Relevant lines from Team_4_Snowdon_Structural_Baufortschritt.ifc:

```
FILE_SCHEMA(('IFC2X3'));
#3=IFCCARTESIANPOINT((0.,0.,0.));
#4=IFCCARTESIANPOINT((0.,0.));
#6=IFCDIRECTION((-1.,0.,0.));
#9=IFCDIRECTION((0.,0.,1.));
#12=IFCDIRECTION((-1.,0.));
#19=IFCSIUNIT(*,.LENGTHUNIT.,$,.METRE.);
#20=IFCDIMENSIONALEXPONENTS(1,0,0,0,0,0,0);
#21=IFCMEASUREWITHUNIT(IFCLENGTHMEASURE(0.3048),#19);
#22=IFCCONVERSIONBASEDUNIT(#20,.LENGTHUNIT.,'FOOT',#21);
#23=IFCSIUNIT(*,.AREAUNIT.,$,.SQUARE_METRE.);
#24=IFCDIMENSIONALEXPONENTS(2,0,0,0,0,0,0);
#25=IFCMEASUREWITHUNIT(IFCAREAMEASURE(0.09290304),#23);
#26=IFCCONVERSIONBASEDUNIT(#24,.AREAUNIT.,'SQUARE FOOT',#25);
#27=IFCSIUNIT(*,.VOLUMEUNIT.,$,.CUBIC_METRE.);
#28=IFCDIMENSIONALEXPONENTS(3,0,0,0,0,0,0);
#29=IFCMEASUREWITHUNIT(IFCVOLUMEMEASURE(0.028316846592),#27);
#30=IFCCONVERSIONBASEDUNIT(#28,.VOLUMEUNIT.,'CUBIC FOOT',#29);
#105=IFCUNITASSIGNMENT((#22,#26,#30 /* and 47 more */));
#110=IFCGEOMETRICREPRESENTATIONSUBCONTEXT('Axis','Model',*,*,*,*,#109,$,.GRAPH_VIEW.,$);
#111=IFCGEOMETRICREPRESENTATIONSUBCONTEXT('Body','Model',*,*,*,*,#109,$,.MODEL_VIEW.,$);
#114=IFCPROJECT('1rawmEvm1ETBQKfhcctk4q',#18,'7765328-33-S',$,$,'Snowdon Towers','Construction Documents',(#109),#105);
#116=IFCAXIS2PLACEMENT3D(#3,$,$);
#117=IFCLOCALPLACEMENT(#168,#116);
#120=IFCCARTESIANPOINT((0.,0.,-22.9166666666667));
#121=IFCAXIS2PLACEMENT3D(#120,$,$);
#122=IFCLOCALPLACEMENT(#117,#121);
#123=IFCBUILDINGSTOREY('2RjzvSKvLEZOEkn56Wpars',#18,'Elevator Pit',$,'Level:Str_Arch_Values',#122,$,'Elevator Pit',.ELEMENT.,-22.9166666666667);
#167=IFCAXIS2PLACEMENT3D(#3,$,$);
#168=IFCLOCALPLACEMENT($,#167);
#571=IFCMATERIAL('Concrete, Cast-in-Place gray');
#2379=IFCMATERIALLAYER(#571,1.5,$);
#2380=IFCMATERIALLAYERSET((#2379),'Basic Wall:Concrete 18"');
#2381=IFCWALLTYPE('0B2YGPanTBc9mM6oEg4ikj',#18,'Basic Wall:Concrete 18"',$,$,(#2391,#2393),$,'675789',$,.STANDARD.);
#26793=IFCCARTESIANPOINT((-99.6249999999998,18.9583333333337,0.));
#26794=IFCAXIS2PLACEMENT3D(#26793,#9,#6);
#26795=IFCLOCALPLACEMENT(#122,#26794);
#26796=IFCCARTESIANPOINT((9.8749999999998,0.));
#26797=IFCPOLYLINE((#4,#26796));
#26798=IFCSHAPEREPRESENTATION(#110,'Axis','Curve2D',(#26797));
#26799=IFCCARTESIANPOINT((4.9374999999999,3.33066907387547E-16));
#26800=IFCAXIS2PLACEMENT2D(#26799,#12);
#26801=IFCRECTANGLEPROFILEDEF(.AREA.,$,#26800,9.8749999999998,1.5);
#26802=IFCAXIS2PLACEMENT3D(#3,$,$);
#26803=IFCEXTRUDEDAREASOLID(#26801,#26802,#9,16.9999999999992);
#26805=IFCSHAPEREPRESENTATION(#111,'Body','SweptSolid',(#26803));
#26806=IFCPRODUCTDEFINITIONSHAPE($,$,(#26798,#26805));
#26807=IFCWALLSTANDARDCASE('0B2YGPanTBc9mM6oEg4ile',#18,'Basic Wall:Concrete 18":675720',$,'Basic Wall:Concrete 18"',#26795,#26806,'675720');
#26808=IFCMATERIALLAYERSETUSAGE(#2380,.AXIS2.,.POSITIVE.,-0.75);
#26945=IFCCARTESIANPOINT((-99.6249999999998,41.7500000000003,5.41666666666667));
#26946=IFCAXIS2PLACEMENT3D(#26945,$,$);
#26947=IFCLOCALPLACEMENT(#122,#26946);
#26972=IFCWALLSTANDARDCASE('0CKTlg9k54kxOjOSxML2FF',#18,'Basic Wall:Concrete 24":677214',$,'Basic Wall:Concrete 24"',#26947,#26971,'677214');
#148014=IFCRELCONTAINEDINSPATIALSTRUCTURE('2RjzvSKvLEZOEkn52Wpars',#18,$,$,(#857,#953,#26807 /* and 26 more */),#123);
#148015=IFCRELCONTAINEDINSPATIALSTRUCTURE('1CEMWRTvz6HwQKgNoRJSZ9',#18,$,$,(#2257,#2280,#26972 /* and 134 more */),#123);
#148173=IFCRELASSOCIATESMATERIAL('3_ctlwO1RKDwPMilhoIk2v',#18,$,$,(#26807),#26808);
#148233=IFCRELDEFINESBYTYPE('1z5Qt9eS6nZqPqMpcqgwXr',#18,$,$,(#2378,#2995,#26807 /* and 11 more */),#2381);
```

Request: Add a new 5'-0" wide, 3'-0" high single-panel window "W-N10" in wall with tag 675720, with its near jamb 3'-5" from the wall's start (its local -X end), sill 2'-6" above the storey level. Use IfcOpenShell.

```python
import numpy as np
import ifcopenshell
import ifcopenshell.api.feature
import ifcopenshell.api.geometry
import ifcopenshell.api.root
import ifcopenshell.api.spatial
import ifcopenshell.api.type
import ifcopenshell.geom
import ifcopenshell.util.element
import ifcopenshell.util.placement
import ifcopenshell.util.representation
import ifcopenshell.util.shape
import ifcopenshell.util.unit

model = ifcopenshell.open("Team_4_Snowdon_Structural_Baufortschritt.ifc")
unit_scale = ifcopenshell.util.unit.calculate_unit_scale(model)
settings = ifcopenshell.geom.settings()


def volume(element):
    """Net volume in cubic metres, openings subtracted."""
    shape = ifcopenshell.geom.create_shape(settings, element)
    return ifcopenshell.util.shape.get_volume(shape.geometry)


wall = model.by_guid("0B2YGPanTBc9mM6oEg4ile")
storey = ifcopenshell.util.element.get_container(wall, ifc_class="IfcBuildingStorey")
context = ifcopenshell.util.representation.get_context(model, "Model", "Body", "MODEL_VIEW")
before = volume(wall)

width, height, from_end, sill = 1.524, 0.9144, 1.0414, 0.762  # metres

# The wall runs along its own X axis, and the end named is its -X end.
wall_shape = ifcopenshell.geom.create_shape(settings, wall)
x, y, z = ifcopenshell.util.shape.get_vertices(wall_shape.geometry).T
start = x.min() + from_end
face, thickness = float(y.min()), float(y.max() - y.min())
wall_matrix = ifcopenshell.util.placement.get_local_placement(wall.ObjectPlacement)
level = ifcopenshell.util.placement.get_local_placement(storey.ObjectPlacement)[2, 3]


def in_wall(x, y):
    """Placement at x, y metres in the wall's axes, at sill height."""
    matrix = wall_matrix.copy()
    matrix[:, 3] = wall_matrix @ np.array([x / unit_scale, y / unit_scale, 0.0, 1.0])
    matrix[2, 3] = level + sill / unit_scale
    return matrix


# Opening: a box that overshoots both wall faces by 50 mm.
opening = ifcopenshell.api.root.create_entity(model, ifc_class="IfcOpeningElement")
box = ifcopenshell.api.geometry.add_wall_representation(
    model, context=context, length=width, height=height, thickness=thickness + 0.1
)
ifcopenshell.api.geometry.assign_representation(model, product=opening, representation=box)
ifcopenshell.api.geometry.edit_object_placement(model, product=opening, matrix=in_wall(start, face - 0.05), is_si=False)
ifcopenshell.api.feature.add_feature(model, feature=opening, element=wall)

window = ifcopenshell.api.root.create_entity(model, ifc_class="IfcWindow", name="W-N10")
window.OverallWidth, window.OverallHeight = width / unit_scale, height / unit_scale
body = ifcopenshell.api.geometry.add_window_representation(
    model,
    context=context,
    overall_width=window.OverallWidth,
    overall_height=window.OverallHeight,
    partition_type="SINGLE_PANEL",
)
ifcopenshell.api.geometry.assign_representation(model, product=window, representation=body)
ifcopenshell.api.spatial.assign_container(model, products=[window], relating_structure=storey)
fills = ifcopenshell.api.feature.add_filling(model, opening=opening, element=window)
fills.OwnerHistory = window.OwnerHistory  # required in IFC2X3

# IFC2X3 keeps the operation on the window style.
style = ifcopenshell.api.root.create_entity(model, ifc_class="IfcWindowStyle", name="W-N10")
style.OperationType, style.ConstructionType = "SINGLE_PANEL", "NOTDEFINED"
style.ParameterTakesPrecedence = style.Sizeable = False
ifcopenshell.api.type.assign_type(model, related_objects=[window], relating_type=style)

# Centre the window in the wall's thickness.
ifcopenshell.api.geometry.edit_object_placement(model, product=window, matrix=in_wall(start, face), is_si=False)
window_shape = ifcopenshell.geom.create_shape(settings, window)
depth = ifcopenshell.util.shape.get_vertices(window_shape.geometry)[:, 1]
offset = face + thickness / 2 - (depth.min() + depth.max()) / 2
ifcopenshell.api.geometry.edit_object_placement(model, product=window, matrix=in_wall(start, offset), is_si=False)

after = volume(wall)

print(f"wall volume {before:.3f} -> {after:.3f} m3")

model.write("Team_4_Snowdon_Structural_Baufortschritt_rev.ifc")
```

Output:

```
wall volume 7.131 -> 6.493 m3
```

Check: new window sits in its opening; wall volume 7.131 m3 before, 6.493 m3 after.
